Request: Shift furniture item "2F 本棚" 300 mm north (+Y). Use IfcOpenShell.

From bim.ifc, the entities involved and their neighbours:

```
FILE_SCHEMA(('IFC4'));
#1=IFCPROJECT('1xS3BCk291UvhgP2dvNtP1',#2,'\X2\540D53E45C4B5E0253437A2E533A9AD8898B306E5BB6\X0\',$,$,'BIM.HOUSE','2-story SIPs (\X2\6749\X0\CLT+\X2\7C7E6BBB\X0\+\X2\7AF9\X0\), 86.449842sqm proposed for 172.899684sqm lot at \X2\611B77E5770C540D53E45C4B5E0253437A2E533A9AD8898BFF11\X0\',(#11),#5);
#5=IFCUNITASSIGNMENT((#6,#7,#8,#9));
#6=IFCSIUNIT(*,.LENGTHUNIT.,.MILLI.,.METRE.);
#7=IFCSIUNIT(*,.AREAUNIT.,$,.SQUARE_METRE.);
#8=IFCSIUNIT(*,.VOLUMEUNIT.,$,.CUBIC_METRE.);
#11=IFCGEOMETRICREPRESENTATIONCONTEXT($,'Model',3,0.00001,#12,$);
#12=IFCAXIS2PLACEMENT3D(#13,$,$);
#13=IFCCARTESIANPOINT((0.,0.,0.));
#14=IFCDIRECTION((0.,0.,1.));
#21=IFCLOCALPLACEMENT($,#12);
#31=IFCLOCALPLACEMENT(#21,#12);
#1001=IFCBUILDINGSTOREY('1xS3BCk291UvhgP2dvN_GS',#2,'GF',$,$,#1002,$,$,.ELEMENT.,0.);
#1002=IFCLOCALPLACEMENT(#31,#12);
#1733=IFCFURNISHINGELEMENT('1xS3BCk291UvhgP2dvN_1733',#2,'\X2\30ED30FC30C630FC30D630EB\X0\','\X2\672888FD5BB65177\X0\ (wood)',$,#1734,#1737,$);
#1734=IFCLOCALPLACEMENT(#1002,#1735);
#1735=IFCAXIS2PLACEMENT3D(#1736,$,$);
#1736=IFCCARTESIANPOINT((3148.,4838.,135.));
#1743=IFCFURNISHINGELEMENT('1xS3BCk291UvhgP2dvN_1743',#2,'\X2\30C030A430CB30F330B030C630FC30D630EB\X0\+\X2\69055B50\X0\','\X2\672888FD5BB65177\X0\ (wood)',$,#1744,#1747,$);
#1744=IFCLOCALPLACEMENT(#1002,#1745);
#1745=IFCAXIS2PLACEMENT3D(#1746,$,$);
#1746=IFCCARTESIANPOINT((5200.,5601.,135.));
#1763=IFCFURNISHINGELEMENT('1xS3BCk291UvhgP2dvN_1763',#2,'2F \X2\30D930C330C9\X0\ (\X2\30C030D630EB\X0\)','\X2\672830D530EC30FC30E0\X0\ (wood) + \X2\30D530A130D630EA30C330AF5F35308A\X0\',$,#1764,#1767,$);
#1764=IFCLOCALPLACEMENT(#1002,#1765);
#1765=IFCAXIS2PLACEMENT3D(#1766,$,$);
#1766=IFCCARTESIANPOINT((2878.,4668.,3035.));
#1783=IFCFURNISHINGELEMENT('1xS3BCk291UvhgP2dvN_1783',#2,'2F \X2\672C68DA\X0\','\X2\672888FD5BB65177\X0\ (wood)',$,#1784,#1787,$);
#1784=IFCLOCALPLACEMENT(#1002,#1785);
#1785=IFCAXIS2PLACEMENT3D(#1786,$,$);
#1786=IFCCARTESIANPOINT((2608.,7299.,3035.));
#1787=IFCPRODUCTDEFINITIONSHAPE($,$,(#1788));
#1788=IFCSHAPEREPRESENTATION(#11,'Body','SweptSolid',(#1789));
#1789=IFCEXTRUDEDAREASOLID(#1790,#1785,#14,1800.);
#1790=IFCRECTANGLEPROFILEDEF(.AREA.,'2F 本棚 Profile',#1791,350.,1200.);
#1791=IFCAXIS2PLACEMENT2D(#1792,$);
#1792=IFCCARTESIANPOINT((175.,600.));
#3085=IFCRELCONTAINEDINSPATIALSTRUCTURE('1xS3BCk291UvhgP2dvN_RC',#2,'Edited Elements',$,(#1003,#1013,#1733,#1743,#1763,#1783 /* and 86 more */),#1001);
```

```python
import ifcopenshell
import ifcopenshell.api.geometry
import ifcopenshell.util.placement
import ifcopenshell.util.unit

model = ifcopenshell.open("bim.ifc")
unit_scale = ifcopenshell.util.unit.calculate_unit_scale(model)

item = model.by_id(1783)
matrix = ifcopenshell.util.placement.get_local_placement(item.ObjectPlacement)
matrix[1, 3] += 0.3 / unit_scale
ifcopenshell.api.geometry.edit_object_placement(model, product=item, matrix=matrix, is_si=False)

print(ifcopenshell.util.placement.get_local_placement(item.ObjectPlacement).round(3) + 0.0)

model.write("bim_edited.ifc")
```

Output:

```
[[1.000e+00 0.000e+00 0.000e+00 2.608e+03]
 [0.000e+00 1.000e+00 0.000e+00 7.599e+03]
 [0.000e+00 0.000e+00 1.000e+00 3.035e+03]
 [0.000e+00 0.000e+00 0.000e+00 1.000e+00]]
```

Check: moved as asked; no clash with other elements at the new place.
